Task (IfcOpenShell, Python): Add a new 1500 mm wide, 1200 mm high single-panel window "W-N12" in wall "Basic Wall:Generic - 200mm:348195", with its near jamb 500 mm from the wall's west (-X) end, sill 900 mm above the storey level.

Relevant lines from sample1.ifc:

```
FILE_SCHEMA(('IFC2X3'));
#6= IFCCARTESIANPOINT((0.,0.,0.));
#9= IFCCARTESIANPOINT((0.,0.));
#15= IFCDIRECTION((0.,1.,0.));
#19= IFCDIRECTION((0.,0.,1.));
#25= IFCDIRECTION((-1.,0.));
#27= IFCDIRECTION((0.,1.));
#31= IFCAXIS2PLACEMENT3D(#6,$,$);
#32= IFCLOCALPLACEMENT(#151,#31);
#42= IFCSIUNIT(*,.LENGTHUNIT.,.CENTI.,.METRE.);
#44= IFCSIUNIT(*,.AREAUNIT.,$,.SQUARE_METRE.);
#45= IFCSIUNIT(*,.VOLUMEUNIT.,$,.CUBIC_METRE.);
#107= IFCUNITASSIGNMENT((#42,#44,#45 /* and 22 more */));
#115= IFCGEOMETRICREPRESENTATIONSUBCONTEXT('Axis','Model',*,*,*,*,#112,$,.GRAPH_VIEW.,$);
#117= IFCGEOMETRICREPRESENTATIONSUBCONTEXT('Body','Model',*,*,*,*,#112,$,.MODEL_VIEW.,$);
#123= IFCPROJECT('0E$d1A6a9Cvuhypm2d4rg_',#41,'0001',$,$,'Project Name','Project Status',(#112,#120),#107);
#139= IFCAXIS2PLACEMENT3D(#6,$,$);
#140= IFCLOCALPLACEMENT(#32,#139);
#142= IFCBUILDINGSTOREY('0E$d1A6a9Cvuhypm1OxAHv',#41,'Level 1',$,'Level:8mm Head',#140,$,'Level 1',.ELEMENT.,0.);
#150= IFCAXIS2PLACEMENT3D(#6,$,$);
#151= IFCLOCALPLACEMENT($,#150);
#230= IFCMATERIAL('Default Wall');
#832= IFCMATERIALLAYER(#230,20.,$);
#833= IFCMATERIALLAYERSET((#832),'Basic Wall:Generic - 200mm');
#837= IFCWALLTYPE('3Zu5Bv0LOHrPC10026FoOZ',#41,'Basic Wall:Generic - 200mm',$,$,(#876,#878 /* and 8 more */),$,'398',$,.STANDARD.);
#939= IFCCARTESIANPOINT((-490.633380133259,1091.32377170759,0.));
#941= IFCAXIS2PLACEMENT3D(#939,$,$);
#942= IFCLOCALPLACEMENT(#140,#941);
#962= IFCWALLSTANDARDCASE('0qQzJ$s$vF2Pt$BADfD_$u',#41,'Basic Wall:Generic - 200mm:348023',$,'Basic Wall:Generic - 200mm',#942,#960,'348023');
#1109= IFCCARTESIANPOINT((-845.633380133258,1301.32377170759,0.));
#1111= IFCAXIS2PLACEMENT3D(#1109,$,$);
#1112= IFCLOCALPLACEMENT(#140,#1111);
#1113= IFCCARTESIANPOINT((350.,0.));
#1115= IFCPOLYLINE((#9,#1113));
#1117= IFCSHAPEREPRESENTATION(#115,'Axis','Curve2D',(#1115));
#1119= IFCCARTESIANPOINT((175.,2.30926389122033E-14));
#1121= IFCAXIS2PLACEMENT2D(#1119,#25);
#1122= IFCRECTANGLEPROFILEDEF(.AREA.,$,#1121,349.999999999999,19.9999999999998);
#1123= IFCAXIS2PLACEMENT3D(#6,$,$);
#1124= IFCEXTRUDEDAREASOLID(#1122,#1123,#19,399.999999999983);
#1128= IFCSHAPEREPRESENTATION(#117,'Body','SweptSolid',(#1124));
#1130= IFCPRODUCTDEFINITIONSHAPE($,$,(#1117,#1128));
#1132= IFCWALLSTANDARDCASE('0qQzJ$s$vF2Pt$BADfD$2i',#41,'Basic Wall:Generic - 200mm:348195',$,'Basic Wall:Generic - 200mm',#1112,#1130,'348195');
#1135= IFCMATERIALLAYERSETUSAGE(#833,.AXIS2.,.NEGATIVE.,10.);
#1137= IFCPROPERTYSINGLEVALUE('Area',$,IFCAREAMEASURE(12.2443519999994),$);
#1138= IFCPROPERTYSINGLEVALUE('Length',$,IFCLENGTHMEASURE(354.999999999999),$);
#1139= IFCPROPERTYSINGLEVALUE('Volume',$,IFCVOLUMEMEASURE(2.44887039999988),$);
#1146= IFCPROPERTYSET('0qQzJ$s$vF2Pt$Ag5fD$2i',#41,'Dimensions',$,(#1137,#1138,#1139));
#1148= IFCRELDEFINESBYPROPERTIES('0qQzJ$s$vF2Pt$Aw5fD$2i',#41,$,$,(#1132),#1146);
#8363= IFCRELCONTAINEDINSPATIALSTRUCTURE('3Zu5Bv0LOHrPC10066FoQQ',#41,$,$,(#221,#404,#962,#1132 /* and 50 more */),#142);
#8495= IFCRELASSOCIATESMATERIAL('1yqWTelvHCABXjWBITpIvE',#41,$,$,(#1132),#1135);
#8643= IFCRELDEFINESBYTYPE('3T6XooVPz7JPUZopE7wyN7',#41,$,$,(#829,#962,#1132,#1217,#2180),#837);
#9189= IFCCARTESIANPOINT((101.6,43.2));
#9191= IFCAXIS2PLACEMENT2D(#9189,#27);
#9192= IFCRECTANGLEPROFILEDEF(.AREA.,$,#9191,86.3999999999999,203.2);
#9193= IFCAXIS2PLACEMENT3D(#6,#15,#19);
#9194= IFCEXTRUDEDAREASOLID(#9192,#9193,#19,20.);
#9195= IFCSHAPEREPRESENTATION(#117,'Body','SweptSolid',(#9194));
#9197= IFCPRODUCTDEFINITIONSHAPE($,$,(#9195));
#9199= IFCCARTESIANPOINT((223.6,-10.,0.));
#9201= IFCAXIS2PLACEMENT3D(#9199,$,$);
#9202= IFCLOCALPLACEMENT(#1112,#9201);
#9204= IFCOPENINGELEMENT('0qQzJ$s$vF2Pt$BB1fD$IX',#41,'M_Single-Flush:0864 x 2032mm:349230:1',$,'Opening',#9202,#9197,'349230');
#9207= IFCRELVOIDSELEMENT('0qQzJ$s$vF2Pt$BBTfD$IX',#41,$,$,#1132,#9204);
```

```python
import numpy as np
import ifcopenshell
import ifcopenshell.api.feature
import ifcopenshell.api.geometry
import ifcopenshell.api.pset
import ifcopenshell.api.root
import ifcopenshell.api.spatial
import ifcopenshell.api.type
import ifcopenshell.geom
import ifcopenshell.util.element
import ifcopenshell.util.placement
import ifcopenshell.util.representation
import ifcopenshell.util.shape
import ifcopenshell.util.unit

model = ifcopenshell.open("sample1.ifc")
unit_scale = ifcopenshell.util.unit.calculate_unit_scale(model)
area_scale = ifcopenshell.util.unit.calculate_unit_scale(model, "AREAUNIT")
volume_scale = ifcopenshell.util.unit.calculate_unit_scale(model, "VOLUMEUNIT")
settings = ifcopenshell.geom.settings()


def volume(element):
    """Net volume in cubic metres, openings subtracted."""
    shape = ifcopenshell.geom.create_shape(settings, element)
    return ifcopenshell.util.shape.get_volume(shape.geometry)


wall = model.by_guid("0qQzJ$s$vF2Pt$BADfD$2i")
storey = ifcopenshell.util.element.get_container(wall, ifc_class="IfcBuildingStorey")
context = ifcopenshell.util.representation.get_context(model, "Model", "Body", "MODEL_VIEW")
before = volume(wall)

width, height, from_end, sill = 1.5, 1.2, 0.5, 0.9  # metres

# The wall runs along its own X axis, and the end named is its -X end.
wall_shape = ifcopenshell.geom.create_shape(settings, wall)
x, y, z = ifcopenshell.util.shape.get_vertices(wall_shape.geometry).T
start = x.min() + from_end
face, thickness = float(y.min()), float(y.max() - y.min())
wall_matrix = ifcopenshell.util.placement.get_local_placement(wall.ObjectPlacement)
level = ifcopenshell.util.placement.get_local_placement(storey.ObjectPlacement)[2, 3]


def in_wall(x, y):
    """Placement at x, y metres in the wall's axes, at sill height."""
    matrix = wall_matrix.copy()
    matrix[:, 3] = wall_matrix @ np.array([x / unit_scale, y / unit_scale, 0.0, 1.0])
    matrix[2, 3] = level + sill / unit_scale
    return matrix


# Opening: a box that overshoots both wall faces by 50 mm.
opening = ifcopenshell.api.root.create_entity(model, ifc_class="IfcOpeningElement")
box = ifcopenshell.api.geometry.add_wall_representation(
    model, context=context, length=width, height=height, thickness=thickness + 0.1
)
ifcopenshell.api.geometry.assign_representation(model, product=opening, representation=box)
ifcopenshell.api.geometry.edit_object_placement(model, product=opening, matrix=in_wall(start, face - 0.05), is_si=False)
ifcopenshell.api.feature.add_feature(model, feature=opening, element=wall)

window = ifcopenshell.api.root.create_entity(model, ifc_class="IfcWindow", name="W-N12")
window.OverallWidth, window.OverallHeight = width / unit_scale, height / unit_scale
body = ifcopenshell.api.geometry.add_window_representation(
    model,
    context=context,
    overall_width=window.OverallWidth,
    overall_height=window.OverallHeight,
    partition_type="SINGLE_PANEL",
)
ifcopenshell.api.geometry.assign_representation(model, product=window, representation=body)
ifcopenshell.api.spatial.assign_container(model, products=[window], relating_structure=storey)
fills = ifcopenshell.api.feature.add_filling(model, opening=opening, element=window)
fills.OwnerHistory = window.OwnerHistory  # required in IFC2X3

# IFC2X3 keeps the operation on the window style.
style = ifcopenshell.api.root.create_entity(model, ifc_class="IfcWindowStyle", name="W-N12")
style.OperationType, style.ConstructionType = "SINGLE_PANEL", "NOTDEFINED"
style.ParameterTakesPrecedence = style.Sizeable = False
ifcopenshell.api.type.assign_type(model, related_objects=[window], relating_type=style)

# Centre the window in the wall's thickness.
ifcopenshell.api.geometry.edit_object_placement(model, product=window, matrix=in_wall(start, face), is_si=False)
window_shape = ifcopenshell.geom.create_shape(settings, window)
depth = ifcopenshell.util.shape.get_vertices(window_shape.geometry)[:, 1]
offset = face + thickness / 2 - (depth.min() + depth.max()) / 2
ifcopenshell.api.geometry.edit_object_placement(model, product=window, matrix=in_wall(start, offset), is_si=False)

after = volume(wall)

# Update the wall's stored quantities.
pset = model.by_id(ifcopenshell.util.element.get_pset(wall, "Dimensions", should_inherit=False)["id"])
ifcopenshell.api.pset.edit_pset(model, pset=pset, properties={
    "Area": model.create_entity("IfcAreaMeasure", after / thickness / area_scale),
    "Volume": model.create_entity("IfcVolumeMeasure", after / volume_scale),
})

print(f"wall volume {before:.3f} -> {after:.3f} m3")

model.write("sample1_edited.ifc")
```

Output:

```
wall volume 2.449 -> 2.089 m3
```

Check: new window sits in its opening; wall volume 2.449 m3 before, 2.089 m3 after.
